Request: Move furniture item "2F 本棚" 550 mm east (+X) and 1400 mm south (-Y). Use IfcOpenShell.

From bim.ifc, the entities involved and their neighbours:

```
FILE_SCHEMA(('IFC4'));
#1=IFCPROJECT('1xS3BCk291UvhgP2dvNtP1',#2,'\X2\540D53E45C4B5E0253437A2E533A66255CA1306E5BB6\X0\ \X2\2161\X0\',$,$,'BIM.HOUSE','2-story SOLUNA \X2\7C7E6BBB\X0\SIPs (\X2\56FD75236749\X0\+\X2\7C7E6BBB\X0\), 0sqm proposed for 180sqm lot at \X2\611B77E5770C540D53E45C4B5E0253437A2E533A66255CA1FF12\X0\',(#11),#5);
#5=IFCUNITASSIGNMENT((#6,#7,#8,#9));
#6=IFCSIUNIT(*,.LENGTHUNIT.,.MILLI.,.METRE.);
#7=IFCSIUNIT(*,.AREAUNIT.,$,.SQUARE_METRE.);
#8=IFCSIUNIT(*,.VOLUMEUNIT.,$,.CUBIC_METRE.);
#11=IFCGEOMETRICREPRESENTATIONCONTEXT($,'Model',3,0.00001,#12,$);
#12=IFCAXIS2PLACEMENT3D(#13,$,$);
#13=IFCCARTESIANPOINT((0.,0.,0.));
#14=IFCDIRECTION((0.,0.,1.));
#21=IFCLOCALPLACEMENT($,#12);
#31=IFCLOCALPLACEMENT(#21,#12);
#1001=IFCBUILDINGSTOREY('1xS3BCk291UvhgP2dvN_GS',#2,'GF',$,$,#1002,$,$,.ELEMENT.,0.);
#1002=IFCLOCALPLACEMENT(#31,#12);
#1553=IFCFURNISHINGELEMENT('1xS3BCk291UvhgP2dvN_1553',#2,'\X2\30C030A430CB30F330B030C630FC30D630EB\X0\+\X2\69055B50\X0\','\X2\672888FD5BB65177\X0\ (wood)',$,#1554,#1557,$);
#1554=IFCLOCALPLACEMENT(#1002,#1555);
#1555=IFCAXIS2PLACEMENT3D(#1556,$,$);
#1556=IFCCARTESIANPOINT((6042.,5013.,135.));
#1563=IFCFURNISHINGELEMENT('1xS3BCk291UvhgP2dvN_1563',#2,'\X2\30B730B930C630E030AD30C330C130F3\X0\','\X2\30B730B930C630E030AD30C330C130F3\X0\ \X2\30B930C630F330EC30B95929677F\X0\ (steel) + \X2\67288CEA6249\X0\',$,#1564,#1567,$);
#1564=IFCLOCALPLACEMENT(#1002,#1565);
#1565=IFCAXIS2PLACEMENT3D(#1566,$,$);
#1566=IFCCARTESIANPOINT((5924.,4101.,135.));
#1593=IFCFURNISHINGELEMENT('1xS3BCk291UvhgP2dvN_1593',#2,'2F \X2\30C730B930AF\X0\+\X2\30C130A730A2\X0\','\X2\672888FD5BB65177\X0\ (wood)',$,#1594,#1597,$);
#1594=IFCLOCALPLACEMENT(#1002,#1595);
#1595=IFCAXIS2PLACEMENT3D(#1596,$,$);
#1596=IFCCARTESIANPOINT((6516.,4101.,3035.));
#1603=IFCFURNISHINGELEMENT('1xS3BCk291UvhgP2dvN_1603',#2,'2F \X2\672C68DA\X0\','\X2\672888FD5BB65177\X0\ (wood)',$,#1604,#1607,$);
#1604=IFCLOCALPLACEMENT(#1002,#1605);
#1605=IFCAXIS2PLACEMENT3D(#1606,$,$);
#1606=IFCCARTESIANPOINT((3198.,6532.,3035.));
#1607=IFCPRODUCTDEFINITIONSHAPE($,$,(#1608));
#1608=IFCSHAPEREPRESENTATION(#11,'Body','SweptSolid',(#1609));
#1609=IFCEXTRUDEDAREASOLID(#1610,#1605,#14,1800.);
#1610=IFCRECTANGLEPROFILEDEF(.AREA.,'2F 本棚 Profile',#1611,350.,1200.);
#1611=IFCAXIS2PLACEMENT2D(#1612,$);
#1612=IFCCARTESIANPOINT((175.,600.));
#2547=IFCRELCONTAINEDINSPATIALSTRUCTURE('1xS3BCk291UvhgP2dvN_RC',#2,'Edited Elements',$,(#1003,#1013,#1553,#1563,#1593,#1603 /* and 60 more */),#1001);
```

```python
import ifcopenshell
import ifcopenshell.api.geometry
import ifcopenshell.util.placement
import ifcopenshell.util.unit

model = ifcopenshell.open("bim.ifc")
unit_scale = ifcopenshell.util.unit.calculate_unit_scale(model)

item = model.by_guid("1xS3BCk291UvhgP2dvN_1603")
matrix = ifcopenshell.util.placement.get_local_placement(item.ObjectPlacement)
matrix[0, 3] += 0.55 / unit_scale
matrix[1, 3] -= 1.4 / unit_scale
ifcopenshell.api.geometry.edit_object_placement(model, product=item, matrix=matrix, is_si=False)

print(ifcopenshell.util.placement.get_local_placement(item.ObjectPlacement).round(3) + 0.0)

model.write("bim_v2.ifc")
```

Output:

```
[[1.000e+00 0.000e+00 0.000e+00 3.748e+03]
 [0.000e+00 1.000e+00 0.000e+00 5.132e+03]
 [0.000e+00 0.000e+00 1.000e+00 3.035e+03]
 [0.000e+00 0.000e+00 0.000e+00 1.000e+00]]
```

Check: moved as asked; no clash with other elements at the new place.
